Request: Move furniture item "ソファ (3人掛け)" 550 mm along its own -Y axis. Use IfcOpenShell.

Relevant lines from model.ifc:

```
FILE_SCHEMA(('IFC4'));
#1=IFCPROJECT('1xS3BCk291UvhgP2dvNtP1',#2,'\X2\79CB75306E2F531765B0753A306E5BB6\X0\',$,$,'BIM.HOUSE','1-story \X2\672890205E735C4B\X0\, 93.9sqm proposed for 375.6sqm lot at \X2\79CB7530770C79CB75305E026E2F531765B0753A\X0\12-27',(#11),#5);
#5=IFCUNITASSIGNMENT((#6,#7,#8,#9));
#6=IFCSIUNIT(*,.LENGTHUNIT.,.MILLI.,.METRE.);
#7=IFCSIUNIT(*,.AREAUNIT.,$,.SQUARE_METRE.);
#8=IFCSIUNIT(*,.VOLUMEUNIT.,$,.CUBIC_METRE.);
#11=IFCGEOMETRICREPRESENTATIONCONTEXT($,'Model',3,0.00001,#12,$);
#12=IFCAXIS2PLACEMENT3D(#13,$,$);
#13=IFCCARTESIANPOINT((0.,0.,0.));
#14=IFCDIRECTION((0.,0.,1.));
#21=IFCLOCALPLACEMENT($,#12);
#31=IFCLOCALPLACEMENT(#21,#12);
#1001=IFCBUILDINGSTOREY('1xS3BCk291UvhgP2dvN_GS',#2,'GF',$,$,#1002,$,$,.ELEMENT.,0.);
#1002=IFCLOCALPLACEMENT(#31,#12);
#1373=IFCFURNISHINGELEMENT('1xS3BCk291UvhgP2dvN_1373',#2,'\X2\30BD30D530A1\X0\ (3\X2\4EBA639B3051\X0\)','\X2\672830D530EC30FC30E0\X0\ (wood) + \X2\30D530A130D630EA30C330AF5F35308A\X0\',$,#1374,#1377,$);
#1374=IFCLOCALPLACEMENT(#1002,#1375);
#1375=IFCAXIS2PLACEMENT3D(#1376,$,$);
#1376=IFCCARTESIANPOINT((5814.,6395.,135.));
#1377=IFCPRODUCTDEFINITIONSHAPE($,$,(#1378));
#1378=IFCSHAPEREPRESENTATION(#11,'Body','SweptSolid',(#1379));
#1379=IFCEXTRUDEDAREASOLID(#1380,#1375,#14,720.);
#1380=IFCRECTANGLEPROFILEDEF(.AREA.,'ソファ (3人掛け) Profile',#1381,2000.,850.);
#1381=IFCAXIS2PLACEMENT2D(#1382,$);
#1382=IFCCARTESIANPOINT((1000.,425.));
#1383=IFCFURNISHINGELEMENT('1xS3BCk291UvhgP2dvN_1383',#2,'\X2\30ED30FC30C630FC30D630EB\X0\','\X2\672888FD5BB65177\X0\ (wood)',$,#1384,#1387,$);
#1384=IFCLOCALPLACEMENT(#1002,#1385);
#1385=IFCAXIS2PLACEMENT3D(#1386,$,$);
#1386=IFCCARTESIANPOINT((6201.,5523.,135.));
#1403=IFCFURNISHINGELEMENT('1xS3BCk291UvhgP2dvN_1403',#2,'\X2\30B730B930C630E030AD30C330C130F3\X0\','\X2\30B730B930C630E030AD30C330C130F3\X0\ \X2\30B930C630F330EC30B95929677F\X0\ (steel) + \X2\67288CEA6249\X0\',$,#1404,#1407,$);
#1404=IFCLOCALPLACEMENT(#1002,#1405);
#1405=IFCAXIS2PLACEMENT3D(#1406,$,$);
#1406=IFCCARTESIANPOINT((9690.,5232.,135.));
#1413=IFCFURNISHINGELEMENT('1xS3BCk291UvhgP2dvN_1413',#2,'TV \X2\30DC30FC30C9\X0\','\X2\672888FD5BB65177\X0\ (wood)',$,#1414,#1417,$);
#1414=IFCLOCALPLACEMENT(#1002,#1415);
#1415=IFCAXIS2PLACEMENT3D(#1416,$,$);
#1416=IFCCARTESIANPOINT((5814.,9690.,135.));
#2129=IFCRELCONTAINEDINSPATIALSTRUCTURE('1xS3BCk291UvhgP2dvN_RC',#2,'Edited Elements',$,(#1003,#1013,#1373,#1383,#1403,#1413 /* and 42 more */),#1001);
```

```python
import ifcopenshell
import ifcopenshell.api.geometry
import ifcopenshell.util.placement
import ifcopenshell.util.unit

model = ifcopenshell.open("model.ifc")
unit_scale = ifcopenshell.util.unit.calculate_unit_scale(model)

item = model.by_id(1373)
matrix = ifcopenshell.util.placement.get_local_placement(item.ObjectPlacement)
matrix[:3, 3] -= matrix[:3, 1] * 0.55 / unit_scale
ifcopenshell.api.geometry.edit_object_placement(model, product=item, matrix=matrix, is_si=False)

print(ifcopenshell.util.placement.get_local_placement(item.ObjectPlacement).round(3) + 0.0)

model.write("model-out.ifc")
```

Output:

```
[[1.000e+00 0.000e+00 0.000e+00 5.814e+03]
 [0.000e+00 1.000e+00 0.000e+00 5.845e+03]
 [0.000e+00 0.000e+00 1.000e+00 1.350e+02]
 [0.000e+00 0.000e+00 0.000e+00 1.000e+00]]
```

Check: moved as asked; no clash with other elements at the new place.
